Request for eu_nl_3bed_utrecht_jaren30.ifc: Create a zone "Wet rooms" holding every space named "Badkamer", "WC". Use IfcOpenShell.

First a look at what the model holds.

```python
import ifcopenshell

model = ifcopenshell.open("eu_nl_3bed_utrecht_jaren30.ifc")
print(model.schema)
seen = {}
for space in model.by_type("IfcSpace"):
    seen[space.LongName] = seen.get(space.LongName, 0) + 1
for name, count in sorted(seen.items(), key=str):
    print(count, "x", name)
print("zones:", [z.Name for z in model.by_type("IfcZone")][:20])
```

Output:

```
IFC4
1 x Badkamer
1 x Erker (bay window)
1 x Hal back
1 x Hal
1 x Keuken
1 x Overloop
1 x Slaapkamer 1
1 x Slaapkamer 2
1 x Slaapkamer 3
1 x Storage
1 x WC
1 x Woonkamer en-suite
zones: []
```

```python
import ifcopenshell
import ifcopenshell.api.group
import ifcopenshell.api.root

model = ifcopenshell.open("eu_nl_3bed_utrecht_jaren30.ifc")

names = {"Badkamer", "WC"}
spaces = [s for s in model.by_type("IfcSpace") if s.LongName in names]

zone = ifcopenshell.api.root.create_entity(model, ifc_class="IfcZone", name="Wet rooms")
ifcopenshell.api.group.assign_group(model, products=spaces, group=zone)
print(len(spaces), "spaces in", zone.Name)

model.write("eu_nl_3bed_utrecht_jaren30-out.ifc")
```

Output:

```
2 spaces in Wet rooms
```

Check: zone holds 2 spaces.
